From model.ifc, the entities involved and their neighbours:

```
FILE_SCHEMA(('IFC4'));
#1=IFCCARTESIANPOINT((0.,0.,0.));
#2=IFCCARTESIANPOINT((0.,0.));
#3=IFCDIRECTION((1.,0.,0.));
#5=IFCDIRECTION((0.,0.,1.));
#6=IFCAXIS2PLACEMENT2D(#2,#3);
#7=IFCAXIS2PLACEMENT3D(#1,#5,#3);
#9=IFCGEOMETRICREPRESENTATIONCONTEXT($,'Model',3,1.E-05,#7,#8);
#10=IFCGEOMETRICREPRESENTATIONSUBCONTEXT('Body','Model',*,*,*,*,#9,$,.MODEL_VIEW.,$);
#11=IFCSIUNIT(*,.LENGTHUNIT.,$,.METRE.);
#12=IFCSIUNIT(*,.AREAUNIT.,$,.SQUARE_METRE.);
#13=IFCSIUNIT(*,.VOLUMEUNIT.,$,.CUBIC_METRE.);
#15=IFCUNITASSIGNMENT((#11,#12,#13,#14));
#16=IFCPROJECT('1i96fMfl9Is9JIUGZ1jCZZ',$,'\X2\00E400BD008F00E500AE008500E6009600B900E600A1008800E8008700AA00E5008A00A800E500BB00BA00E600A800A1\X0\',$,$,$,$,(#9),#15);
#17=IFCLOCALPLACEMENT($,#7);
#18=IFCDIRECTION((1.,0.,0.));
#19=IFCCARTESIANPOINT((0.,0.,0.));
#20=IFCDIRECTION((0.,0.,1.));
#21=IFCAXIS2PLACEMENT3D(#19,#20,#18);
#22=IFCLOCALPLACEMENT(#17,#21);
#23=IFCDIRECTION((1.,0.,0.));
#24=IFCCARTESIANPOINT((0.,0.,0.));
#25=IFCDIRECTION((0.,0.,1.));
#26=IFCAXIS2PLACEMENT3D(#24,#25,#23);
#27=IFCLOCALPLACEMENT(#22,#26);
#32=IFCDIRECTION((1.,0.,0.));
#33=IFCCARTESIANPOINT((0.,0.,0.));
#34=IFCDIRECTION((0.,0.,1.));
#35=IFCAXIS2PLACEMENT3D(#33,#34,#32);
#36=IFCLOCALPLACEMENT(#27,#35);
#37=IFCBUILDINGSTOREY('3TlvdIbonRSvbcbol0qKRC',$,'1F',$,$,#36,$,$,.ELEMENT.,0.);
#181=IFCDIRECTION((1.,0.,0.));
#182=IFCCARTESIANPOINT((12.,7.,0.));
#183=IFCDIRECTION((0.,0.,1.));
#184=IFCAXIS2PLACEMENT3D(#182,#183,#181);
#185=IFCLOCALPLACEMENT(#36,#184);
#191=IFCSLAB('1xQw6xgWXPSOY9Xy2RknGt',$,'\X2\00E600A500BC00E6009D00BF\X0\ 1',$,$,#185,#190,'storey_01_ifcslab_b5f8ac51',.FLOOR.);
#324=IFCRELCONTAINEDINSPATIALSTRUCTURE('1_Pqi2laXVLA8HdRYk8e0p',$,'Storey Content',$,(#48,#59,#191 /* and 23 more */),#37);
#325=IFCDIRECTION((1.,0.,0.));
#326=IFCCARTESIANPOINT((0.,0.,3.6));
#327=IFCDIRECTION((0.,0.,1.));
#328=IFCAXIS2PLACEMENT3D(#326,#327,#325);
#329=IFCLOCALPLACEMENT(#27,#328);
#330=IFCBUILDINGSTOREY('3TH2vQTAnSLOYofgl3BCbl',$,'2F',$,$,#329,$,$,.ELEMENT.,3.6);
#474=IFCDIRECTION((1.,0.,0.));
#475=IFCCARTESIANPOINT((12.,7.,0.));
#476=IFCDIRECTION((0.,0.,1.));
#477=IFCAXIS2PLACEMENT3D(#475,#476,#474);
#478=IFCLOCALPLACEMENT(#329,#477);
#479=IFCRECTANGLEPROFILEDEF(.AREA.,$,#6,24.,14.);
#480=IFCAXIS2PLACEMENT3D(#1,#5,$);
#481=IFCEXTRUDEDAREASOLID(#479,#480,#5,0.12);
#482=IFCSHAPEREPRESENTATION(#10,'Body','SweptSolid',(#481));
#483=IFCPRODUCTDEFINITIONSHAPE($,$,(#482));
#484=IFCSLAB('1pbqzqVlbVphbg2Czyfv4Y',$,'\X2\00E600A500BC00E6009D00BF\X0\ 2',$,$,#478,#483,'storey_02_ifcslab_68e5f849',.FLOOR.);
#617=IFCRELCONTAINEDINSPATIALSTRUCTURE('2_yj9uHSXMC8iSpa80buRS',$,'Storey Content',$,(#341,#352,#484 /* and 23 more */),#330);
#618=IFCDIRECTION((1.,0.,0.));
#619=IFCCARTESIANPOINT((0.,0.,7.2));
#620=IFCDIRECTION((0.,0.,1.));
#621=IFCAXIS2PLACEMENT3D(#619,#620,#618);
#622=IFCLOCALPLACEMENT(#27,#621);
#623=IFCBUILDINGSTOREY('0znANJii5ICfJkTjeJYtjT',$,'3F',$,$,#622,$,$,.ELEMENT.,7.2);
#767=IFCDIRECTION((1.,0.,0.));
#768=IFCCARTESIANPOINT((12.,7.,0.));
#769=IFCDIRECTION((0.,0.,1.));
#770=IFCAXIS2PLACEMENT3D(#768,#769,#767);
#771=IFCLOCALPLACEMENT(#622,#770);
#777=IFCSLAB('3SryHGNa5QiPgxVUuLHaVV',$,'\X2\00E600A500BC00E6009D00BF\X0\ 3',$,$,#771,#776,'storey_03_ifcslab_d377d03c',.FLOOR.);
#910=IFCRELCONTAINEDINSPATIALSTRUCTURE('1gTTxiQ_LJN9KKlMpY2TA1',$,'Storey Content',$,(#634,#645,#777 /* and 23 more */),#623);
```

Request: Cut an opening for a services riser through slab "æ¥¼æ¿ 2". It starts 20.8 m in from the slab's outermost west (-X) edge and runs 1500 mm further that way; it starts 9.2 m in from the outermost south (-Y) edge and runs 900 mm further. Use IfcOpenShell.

```python
import numpy as np
import ifcopenshell
import ifcopenshell.api.feature
import ifcopenshell.api.geometry
import ifcopenshell.api.root
import ifcopenshell.geom
import ifcopenshell.util.placement
import ifcopenshell.util.representation
import ifcopenshell.util.shape
import ifcopenshell.util.unit

model = ifcopenshell.open("model.ifc")
unit_scale = ifcopenshell.util.unit.calculate_unit_scale(model)
settings = ifcopenshell.geom.settings()


def volume(element):
    """Net volume in cubic metres, openings subtracted."""
    shape = ifcopenshell.geom.create_shape(settings, element)
    return ifcopenshell.util.shape.get_volume(shape.geometry)


slab = model.by_guid("1pbqzqVlbVphbg2Czyfv4Y")
before = volume(slab)

# Extent in the slab's own axes, in metres. The edges named are its -X and -Y sides.
slab_shape = ifcopenshell.geom.create_shape(settings, slab)
vertices = ifcopenshell.util.shape.get_vertices(slab_shape.geometry)
x_min, y_min, bottom = vertices.min(axis=0)
top = vertices[:, 2].max()

opening = ifcopenshell.api.root.create_entity(model, ifc_class="IfcOpeningElement", name="Services riser opening", predefined_type="OPENING")
context = ifcopenshell.util.representation.get_context(model, "Model", "Body", "MODEL_VIEW")
width, depth = 1.5, 0.9
outline = [(0.0, 0.0), (width, 0.0), (width, depth), (0.0, depth), (0.0, 0.0)]
# Overshoot both faces by 50 mm so the cut is clean.
shape = ifcopenshell.api.geometry.add_slab_representation(
    model, context=context, depth=top - bottom + 0.1, polyline=outline
)
ifcopenshell.api.geometry.assign_representation(model, product=opening, representation=shape)

matrix = ifcopenshell.util.placement.get_local_placement(slab.ObjectPlacement)
matrix[:, 3] = matrix @ np.append(np.array([x_min + 20.8, y_min + 9.2, bottom - 0.05]) / unit_scale, 1.0)
ifcopenshell.api.geometry.edit_object_placement(model, product=opening, matrix=matrix, is_si=False)
ifcopenshell.api.feature.add_feature(model, feature=opening, element=slab)

after = volume(slab)

print(f"slab volume {before:.3f} -> {after:.3f} m3")

model.write("model-out.ifc")
```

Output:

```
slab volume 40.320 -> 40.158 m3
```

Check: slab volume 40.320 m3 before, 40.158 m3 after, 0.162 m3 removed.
